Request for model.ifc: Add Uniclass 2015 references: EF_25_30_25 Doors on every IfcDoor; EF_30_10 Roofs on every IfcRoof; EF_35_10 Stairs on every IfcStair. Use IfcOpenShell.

First a look at what the model holds.

```python
import ifcopenshell

model = ifcopenshell.open("model.ifc")
print(model.schema)
print("classifications:", [c.Name for c in model.by_type("IfcClassification")])
for ifc_class in ("IfcDoor", "IfcRoof", "IfcStair", "IfcWall", "IfcWindow"):
    print(ifc_class, len(model.by_type(ifc_class)))
```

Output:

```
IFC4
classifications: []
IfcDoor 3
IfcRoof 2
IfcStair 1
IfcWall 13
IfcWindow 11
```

```python
import ifcopenshell
import ifcopenshell.api.classification

model = ifcopenshell.open("model.ifc")

system = ifcopenshell.api.classification.add_classification(model, classification="Uniclass 2015")

codes = {
    "IfcDoor": ("EF_25_30_25", "Doors"),
    "IfcRoof": ("EF_30_10", "Roofs"),
    "IfcStair": ("EF_35_10", "Stairs"),
}
for ifc_class, (code, name) in codes.items():
    products = model.by_type(ifc_class)
    ifcopenshell.api.classification.add_reference(
        model, products=products, classification=system, identification=code, name=name
    )
    print(code, len(products))

model.write("model_v2.ifc")
```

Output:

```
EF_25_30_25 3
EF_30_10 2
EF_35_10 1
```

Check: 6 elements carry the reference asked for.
